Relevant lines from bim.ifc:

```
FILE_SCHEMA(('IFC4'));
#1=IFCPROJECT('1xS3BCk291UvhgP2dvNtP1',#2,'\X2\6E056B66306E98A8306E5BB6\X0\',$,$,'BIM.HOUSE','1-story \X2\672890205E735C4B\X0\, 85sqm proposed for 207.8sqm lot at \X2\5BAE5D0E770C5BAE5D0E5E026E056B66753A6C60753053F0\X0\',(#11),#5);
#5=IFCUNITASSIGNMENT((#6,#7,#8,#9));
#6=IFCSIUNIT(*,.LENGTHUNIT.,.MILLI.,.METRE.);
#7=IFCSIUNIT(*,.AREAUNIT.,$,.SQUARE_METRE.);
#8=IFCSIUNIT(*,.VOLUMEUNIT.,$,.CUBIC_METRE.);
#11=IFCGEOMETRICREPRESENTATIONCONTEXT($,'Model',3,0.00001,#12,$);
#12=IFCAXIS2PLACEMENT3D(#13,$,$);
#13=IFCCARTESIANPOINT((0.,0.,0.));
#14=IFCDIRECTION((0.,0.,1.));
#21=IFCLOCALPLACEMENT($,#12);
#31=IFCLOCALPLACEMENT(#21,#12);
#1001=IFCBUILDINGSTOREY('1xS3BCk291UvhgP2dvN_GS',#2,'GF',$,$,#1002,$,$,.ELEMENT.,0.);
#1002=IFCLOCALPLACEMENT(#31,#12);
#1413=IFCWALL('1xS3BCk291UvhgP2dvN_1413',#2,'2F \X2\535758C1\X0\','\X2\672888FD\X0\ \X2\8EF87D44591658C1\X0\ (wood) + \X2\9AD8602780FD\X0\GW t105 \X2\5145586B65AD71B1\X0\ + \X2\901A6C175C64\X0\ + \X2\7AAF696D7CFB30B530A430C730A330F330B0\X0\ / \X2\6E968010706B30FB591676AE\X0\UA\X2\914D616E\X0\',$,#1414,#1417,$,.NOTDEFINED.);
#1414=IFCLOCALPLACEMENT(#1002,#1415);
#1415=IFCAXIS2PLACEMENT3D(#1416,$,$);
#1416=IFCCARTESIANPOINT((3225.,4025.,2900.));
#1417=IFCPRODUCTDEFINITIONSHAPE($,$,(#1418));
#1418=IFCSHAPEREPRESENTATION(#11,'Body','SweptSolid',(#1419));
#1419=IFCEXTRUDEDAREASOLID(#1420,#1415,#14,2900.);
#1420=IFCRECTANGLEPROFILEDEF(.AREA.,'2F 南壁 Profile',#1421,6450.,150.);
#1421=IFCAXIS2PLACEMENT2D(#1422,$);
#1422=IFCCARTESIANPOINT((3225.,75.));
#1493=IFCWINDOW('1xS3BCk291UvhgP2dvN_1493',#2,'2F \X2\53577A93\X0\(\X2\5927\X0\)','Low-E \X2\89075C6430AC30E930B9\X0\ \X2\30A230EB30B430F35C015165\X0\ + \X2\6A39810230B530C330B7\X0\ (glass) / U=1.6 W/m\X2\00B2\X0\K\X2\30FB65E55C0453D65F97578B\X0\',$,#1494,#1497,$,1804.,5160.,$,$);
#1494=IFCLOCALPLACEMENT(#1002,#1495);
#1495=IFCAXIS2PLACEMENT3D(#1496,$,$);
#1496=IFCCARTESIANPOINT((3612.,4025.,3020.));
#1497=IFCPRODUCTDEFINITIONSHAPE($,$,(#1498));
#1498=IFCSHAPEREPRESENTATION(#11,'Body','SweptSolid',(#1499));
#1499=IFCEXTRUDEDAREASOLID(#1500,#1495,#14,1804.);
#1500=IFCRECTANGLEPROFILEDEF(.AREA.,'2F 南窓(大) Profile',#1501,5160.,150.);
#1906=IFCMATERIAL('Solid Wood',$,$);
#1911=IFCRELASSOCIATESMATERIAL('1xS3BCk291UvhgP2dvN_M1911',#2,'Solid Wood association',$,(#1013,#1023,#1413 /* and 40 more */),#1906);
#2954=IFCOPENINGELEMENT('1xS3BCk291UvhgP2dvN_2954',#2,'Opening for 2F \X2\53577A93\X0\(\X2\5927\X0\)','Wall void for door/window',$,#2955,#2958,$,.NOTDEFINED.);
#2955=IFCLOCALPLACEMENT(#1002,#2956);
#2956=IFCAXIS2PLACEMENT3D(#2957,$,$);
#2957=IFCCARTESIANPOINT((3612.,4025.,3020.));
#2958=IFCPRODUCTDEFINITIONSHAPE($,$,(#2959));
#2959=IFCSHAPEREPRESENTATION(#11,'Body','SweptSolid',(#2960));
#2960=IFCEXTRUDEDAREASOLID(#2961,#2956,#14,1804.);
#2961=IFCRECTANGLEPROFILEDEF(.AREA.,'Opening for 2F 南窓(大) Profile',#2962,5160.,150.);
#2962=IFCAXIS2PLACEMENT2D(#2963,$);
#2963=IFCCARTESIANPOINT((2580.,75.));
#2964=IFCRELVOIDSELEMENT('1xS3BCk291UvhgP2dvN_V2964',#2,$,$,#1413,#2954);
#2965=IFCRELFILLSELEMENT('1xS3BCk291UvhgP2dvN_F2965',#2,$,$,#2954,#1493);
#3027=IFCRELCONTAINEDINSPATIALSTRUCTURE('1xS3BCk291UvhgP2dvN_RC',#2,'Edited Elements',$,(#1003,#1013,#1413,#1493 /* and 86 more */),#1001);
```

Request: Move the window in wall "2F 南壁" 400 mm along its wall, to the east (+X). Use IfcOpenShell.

```python
import ifcopenshell
import ifcopenshell.api.geometry
import ifcopenshell.util.placement

model = ifcopenshell.open("bim.ifc")

window = model.by_id(1493)
opening = window.FillsVoids[0].RelatingOpeningElement
wall = opening.VoidsElements[0].RelatingBuildingElement

wall_matrix = ifcopenshell.util.placement.get_local_placement(wall.ObjectPlacement)
shift = wall_matrix[:3, 0] * 400.0
before = ifcopenshell.util.placement.get_local_placement(window.ObjectPlacement)[:3, 3].copy()

# The window is not placed relative to its opening, so move both.
for product in (opening, window):
    matrix = ifcopenshell.util.placement.get_local_placement(product.ObjectPlacement)
    matrix[:3, 3] += shift
    ifcopenshell.api.geometry.edit_object_placement(model, product=product, matrix=matrix, is_si=False)

after = ifcopenshell.util.placement.get_local_placement(window.ObjectPlacement)[:3, 3]
print("window moved by", (after - before).round(3) + 0.0)

model.write("bim_updated.ifc")
```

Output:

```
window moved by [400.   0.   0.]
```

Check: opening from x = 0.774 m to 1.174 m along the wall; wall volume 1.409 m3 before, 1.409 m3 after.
